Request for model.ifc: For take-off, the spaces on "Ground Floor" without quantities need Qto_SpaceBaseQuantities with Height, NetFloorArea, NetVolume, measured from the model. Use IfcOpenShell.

First a look at what the model holds.

```python
import ifcopenshell
import ifcopenshell.util.element
import ifcopenshell.util.unit

model = ifcopenshell.open("model.ifc")
print(model.schema)
for unit_type in ("LENGTHUNIT", "AREAUNIT", "VOLUMEUNIT"):
    print(unit_type, ifcopenshell.util.unit.calculate_unit_scale(model, unit_type))
storey = next(s for s in model.by_type("IfcBuildingStorey") if s.Name == "Ground Floor")
spaces = [e for e in ifcopenshell.util.element.get_decomposition(storey) if e.is_a("IfcSpace")]
for e in sorted(spaces, key=lambda e: e.id()):
    print(e.id(), e.is_a(), e.Name, list(ifcopenshell.util.element.get_psets(e, qtos_only=True)), sep=" | ")
```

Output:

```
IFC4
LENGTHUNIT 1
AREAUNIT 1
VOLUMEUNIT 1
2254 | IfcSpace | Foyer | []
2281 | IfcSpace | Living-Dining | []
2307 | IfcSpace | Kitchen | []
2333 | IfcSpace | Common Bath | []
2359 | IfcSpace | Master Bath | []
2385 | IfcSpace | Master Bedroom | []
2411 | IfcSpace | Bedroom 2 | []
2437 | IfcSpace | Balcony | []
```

```python
import ifcopenshell
import ifcopenshell.api.pset
import ifcopenshell.geom
import ifcopenshell.util.element
import ifcopenshell.util.shape
import ifcopenshell.util.unit

model = ifcopenshell.open("model.ifc")
unit_scale = ifcopenshell.util.unit.calculate_unit_scale(model)
area_scale = ifcopenshell.util.unit.calculate_unit_scale(model, "AREAUNIT")
volume_scale = ifcopenshell.util.unit.calculate_unit_scale(model, "VOLUMEUNIT")
settings = ifcopenshell.geom.settings()

storey = next(s for s in model.by_type("IfcBuildingStorey") if s.Name == "Ground Floor")
spaces = [e for e in ifcopenshell.util.element.get_decomposition(storey) if e.is_a("IfcSpace")]

for e in sorted(spaces, key=lambda e: e.id()):
    if ifcopenshell.util.element.get_psets(e, qtos_only=True, should_inherit=False):
        continue
    # Geometry comes back in metres, in the element's own axes.
    shape = ifcopenshell.geom.create_shape(settings, e)
    values = {
        "Height": ifcopenshell.util.shape.get_z(shape.geometry) / unit_scale,
        "NetFloorArea": ifcopenshell.util.shape.get_footprint_area(shape.geometry) / area_scale,
        "NetVolume": ifcopenshell.util.shape.get_volume(shape.geometry) / volume_scale,
    }
    qto = ifcopenshell.api.pset.add_qto(model, product=e, name="Qto_SpaceBaseQuantities")
    ifcopenshell.api.pset.edit_qto(model, qto=qto, properties=values)
    print(e.id(), {k: round(v, 3) for k, v in values.items()})

model.write("model_v2.ifc")
```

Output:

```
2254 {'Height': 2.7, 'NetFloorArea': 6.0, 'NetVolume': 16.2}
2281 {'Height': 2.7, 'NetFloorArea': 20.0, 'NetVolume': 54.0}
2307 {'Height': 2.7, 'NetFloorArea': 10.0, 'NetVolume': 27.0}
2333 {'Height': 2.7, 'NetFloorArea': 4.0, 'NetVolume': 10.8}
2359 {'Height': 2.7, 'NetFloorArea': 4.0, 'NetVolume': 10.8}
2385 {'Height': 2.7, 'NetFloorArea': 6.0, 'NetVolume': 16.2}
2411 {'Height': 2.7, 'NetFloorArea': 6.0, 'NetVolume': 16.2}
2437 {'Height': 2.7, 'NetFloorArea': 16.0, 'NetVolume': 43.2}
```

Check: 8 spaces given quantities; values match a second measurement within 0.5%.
